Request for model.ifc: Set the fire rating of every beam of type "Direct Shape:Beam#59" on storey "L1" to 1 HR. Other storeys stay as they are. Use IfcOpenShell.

First a look at what the model holds.

```python
import ifcopenshell
import ifcopenshell.util.element

model = ifcopenshell.open("model.ifc")
print(model.schema)
storey = next(s for s in model.by_type("IfcBuildingStorey") if s.Name == "L1")
beams = [e for e in ifcopenshell.util.element.get_decomposition(storey) if e.is_a("IfcBeam")]
seen = {}
for e in beams:
    element_type = ifcopenshell.util.element.get_type(e)
    key = (element_type.Name if element_type != e and element_type else None, ifcopenshell.util.element.get_pset(e, "Pset_BeamCommon", "FireRating"))
    seen[key] = seen.get(key, 0) + 1
for (name, value), count in sorted(seen.items(), key=str):
    print(count, "x", name, "|", value)
```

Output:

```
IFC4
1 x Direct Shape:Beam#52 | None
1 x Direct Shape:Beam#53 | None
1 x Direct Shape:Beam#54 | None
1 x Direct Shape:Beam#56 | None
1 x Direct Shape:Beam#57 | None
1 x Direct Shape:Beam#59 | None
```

```python
import ifcopenshell
import ifcopenshell.api.pset
import ifcopenshell.util.element

model = ifcopenshell.open("model.ifc")

storey = next(s for s in model.by_type("IfcBuildingStorey") if s.Name == "L1")
beams = [e for e in ifcopenshell.util.element.get_decomposition(storey) if e.is_a("IfcBeam")]

count = 0
for e in beams:
    element_type = ifcopenshell.util.element.get_type(e)
    if element_type in (None, e) or element_type.Name != "Direct Shape:Beam#59":
        continue
    # add_pset returns the element's existing set when there is one.
    pset = ifcopenshell.api.pset.add_pset(model, product=e, name="Pset_BeamCommon")
    ifcopenshell.api.pset.edit_pset(model, pset=pset, properties={"FireRating": "1 HR"})
    count += 1

print(count, "beams updated")

model.write("model_rev.ifc")
```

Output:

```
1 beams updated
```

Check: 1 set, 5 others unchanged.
